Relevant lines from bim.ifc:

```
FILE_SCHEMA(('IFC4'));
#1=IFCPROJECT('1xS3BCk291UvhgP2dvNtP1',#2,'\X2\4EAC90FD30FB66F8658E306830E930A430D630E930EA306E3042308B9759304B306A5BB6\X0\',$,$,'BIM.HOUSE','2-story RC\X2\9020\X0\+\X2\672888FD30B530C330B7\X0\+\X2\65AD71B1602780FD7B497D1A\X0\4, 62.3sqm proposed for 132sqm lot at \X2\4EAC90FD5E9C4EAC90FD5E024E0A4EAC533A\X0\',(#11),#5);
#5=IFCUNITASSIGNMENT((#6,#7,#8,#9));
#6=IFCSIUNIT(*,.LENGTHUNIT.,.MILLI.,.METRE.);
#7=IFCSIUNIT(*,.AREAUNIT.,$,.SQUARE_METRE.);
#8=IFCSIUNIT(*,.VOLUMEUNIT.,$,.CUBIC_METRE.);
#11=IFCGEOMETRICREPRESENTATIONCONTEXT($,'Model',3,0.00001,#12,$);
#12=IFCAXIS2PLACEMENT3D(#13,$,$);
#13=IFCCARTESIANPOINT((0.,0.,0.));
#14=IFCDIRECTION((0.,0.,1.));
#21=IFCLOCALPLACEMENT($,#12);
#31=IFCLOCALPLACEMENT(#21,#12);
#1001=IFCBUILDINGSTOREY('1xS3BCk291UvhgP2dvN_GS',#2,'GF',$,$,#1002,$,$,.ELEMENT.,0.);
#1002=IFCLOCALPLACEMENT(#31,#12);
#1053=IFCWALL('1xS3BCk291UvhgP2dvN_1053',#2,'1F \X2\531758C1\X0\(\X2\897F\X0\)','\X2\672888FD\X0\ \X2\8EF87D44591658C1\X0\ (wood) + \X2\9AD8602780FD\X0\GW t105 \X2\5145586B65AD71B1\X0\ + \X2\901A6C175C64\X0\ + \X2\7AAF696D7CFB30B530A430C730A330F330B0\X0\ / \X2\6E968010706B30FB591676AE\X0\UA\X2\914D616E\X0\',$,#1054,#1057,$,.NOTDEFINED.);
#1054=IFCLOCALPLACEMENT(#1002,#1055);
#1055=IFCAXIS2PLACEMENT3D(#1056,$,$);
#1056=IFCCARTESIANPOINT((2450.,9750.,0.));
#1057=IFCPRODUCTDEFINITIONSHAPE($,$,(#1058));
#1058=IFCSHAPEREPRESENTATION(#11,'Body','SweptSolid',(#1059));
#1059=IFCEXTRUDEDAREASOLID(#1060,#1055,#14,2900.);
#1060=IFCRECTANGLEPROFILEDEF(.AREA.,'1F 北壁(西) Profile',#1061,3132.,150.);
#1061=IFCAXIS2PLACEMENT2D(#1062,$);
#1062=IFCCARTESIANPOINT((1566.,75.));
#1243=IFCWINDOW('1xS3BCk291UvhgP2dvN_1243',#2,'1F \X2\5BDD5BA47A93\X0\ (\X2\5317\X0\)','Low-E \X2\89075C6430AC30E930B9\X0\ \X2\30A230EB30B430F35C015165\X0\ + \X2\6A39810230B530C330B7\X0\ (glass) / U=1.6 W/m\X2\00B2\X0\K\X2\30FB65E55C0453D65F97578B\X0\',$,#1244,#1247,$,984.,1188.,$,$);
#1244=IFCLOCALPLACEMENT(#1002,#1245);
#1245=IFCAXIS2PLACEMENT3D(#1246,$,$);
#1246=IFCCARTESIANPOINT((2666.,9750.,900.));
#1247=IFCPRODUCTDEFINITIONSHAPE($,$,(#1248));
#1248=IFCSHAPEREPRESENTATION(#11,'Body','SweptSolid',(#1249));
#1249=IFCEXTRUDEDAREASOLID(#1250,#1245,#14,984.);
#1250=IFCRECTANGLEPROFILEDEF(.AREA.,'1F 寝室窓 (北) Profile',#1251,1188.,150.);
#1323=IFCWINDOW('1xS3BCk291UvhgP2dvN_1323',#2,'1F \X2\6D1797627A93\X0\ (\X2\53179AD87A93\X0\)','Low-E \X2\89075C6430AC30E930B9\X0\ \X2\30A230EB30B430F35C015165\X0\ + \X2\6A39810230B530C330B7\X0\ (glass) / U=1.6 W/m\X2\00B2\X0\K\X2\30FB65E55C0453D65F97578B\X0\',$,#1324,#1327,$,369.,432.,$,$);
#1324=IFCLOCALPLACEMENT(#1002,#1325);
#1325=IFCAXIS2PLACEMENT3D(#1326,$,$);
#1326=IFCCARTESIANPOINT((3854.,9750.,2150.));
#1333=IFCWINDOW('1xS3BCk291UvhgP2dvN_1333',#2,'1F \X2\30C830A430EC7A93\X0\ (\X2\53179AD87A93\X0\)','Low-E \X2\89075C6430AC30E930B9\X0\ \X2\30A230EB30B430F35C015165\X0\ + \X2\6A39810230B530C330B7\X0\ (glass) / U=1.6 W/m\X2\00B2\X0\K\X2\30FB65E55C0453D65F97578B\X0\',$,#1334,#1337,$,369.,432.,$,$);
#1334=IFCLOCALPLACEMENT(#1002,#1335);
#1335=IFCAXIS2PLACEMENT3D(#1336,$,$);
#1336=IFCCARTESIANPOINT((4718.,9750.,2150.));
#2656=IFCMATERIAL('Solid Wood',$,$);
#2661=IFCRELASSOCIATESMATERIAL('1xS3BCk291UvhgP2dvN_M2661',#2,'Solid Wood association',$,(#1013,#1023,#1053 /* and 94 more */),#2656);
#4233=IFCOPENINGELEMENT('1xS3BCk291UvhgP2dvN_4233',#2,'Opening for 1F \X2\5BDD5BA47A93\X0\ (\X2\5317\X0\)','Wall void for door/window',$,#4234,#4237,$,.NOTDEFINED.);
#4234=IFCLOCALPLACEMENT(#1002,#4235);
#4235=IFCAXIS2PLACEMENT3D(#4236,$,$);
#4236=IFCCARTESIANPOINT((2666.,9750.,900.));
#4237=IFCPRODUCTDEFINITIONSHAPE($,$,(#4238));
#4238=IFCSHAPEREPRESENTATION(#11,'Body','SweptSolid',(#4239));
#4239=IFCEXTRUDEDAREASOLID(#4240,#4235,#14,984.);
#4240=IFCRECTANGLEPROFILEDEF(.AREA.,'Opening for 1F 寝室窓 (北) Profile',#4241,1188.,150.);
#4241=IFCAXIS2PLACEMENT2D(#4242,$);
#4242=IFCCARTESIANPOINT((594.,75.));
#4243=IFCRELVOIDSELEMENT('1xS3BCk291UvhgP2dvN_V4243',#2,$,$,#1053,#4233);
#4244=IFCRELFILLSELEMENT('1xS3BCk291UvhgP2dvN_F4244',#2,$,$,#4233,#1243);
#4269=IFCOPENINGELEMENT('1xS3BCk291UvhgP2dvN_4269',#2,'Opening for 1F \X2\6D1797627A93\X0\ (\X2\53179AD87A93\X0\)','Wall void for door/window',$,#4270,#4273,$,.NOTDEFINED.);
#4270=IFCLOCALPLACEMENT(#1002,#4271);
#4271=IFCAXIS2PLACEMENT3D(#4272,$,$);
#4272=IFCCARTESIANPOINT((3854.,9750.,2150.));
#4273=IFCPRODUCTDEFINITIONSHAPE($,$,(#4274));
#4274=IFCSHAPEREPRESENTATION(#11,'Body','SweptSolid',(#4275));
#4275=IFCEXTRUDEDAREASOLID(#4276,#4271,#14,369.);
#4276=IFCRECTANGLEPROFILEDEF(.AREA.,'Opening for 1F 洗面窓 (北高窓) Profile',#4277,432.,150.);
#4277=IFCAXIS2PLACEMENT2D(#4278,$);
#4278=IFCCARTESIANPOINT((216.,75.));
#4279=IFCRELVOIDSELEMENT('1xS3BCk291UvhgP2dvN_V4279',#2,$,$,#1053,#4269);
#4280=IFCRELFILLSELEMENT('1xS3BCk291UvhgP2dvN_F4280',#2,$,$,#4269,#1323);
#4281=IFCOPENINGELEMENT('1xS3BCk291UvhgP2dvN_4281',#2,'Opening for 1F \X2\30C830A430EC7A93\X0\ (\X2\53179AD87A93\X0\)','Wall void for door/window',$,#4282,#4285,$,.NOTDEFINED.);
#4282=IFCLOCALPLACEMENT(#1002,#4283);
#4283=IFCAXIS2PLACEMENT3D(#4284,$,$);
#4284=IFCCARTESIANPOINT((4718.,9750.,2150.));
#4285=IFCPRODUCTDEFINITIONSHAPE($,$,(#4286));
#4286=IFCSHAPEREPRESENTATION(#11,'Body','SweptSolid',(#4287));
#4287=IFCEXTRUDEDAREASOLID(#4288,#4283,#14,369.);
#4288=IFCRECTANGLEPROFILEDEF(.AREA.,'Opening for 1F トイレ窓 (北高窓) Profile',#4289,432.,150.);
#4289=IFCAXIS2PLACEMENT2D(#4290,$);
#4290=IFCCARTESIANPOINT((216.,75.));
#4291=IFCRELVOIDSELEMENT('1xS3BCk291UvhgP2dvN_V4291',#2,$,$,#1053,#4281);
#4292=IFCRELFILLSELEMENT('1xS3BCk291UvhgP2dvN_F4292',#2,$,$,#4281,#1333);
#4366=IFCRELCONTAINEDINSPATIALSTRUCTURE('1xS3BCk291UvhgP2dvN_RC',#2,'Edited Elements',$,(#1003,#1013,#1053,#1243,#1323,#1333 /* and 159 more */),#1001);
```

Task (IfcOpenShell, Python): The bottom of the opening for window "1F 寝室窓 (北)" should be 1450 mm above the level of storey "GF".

```python
import numpy as np
import ifcopenshell
import ifcopenshell.api.geometry
import ifcopenshell.geom
import ifcopenshell.util.element
import ifcopenshell.util.placement
import ifcopenshell.util.shape
import ifcopenshell.util.unit

model = ifcopenshell.open("bim.ifc")
unit_scale = ifcopenshell.util.unit.calculate_unit_scale(model)

window = model.by_id(1243)
opening = window.FillsVoids[0].RelatingOpeningElement
storey = ifcopenshell.util.element.get_container(window, ifc_class="IfcBuildingStorey")
level = ifcopenshell.util.placement.get_local_placement(storey.ObjectPlacement)[2, 3]

# The opening's origin need not be at the sill, so measure its lowest point.
shape = ifcopenshell.geom.create_shape(ifcopenshell.geom.settings(), opening)
bottom = ifcopenshell.util.shape.get_shape_bottom_elevation(shape, shape.geometry) / unit_scale
dz = level + 1450.0 - bottom

shift = np.array([0.0, 0.0, dz])
# The window is not placed relative to its opening, so move both.
for product in (opening, window):
    matrix = ifcopenshell.util.placement.get_local_placement(product.ObjectPlacement)
    matrix[:3, 3] += shift
    ifcopenshell.api.geometry.edit_object_placement(model, product=product, matrix=matrix, is_si=False)

print(f"moved by {dz * unit_scale:+.3f} m")

model.write("bim_updated.ifc")
```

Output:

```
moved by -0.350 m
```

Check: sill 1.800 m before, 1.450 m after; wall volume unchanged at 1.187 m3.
